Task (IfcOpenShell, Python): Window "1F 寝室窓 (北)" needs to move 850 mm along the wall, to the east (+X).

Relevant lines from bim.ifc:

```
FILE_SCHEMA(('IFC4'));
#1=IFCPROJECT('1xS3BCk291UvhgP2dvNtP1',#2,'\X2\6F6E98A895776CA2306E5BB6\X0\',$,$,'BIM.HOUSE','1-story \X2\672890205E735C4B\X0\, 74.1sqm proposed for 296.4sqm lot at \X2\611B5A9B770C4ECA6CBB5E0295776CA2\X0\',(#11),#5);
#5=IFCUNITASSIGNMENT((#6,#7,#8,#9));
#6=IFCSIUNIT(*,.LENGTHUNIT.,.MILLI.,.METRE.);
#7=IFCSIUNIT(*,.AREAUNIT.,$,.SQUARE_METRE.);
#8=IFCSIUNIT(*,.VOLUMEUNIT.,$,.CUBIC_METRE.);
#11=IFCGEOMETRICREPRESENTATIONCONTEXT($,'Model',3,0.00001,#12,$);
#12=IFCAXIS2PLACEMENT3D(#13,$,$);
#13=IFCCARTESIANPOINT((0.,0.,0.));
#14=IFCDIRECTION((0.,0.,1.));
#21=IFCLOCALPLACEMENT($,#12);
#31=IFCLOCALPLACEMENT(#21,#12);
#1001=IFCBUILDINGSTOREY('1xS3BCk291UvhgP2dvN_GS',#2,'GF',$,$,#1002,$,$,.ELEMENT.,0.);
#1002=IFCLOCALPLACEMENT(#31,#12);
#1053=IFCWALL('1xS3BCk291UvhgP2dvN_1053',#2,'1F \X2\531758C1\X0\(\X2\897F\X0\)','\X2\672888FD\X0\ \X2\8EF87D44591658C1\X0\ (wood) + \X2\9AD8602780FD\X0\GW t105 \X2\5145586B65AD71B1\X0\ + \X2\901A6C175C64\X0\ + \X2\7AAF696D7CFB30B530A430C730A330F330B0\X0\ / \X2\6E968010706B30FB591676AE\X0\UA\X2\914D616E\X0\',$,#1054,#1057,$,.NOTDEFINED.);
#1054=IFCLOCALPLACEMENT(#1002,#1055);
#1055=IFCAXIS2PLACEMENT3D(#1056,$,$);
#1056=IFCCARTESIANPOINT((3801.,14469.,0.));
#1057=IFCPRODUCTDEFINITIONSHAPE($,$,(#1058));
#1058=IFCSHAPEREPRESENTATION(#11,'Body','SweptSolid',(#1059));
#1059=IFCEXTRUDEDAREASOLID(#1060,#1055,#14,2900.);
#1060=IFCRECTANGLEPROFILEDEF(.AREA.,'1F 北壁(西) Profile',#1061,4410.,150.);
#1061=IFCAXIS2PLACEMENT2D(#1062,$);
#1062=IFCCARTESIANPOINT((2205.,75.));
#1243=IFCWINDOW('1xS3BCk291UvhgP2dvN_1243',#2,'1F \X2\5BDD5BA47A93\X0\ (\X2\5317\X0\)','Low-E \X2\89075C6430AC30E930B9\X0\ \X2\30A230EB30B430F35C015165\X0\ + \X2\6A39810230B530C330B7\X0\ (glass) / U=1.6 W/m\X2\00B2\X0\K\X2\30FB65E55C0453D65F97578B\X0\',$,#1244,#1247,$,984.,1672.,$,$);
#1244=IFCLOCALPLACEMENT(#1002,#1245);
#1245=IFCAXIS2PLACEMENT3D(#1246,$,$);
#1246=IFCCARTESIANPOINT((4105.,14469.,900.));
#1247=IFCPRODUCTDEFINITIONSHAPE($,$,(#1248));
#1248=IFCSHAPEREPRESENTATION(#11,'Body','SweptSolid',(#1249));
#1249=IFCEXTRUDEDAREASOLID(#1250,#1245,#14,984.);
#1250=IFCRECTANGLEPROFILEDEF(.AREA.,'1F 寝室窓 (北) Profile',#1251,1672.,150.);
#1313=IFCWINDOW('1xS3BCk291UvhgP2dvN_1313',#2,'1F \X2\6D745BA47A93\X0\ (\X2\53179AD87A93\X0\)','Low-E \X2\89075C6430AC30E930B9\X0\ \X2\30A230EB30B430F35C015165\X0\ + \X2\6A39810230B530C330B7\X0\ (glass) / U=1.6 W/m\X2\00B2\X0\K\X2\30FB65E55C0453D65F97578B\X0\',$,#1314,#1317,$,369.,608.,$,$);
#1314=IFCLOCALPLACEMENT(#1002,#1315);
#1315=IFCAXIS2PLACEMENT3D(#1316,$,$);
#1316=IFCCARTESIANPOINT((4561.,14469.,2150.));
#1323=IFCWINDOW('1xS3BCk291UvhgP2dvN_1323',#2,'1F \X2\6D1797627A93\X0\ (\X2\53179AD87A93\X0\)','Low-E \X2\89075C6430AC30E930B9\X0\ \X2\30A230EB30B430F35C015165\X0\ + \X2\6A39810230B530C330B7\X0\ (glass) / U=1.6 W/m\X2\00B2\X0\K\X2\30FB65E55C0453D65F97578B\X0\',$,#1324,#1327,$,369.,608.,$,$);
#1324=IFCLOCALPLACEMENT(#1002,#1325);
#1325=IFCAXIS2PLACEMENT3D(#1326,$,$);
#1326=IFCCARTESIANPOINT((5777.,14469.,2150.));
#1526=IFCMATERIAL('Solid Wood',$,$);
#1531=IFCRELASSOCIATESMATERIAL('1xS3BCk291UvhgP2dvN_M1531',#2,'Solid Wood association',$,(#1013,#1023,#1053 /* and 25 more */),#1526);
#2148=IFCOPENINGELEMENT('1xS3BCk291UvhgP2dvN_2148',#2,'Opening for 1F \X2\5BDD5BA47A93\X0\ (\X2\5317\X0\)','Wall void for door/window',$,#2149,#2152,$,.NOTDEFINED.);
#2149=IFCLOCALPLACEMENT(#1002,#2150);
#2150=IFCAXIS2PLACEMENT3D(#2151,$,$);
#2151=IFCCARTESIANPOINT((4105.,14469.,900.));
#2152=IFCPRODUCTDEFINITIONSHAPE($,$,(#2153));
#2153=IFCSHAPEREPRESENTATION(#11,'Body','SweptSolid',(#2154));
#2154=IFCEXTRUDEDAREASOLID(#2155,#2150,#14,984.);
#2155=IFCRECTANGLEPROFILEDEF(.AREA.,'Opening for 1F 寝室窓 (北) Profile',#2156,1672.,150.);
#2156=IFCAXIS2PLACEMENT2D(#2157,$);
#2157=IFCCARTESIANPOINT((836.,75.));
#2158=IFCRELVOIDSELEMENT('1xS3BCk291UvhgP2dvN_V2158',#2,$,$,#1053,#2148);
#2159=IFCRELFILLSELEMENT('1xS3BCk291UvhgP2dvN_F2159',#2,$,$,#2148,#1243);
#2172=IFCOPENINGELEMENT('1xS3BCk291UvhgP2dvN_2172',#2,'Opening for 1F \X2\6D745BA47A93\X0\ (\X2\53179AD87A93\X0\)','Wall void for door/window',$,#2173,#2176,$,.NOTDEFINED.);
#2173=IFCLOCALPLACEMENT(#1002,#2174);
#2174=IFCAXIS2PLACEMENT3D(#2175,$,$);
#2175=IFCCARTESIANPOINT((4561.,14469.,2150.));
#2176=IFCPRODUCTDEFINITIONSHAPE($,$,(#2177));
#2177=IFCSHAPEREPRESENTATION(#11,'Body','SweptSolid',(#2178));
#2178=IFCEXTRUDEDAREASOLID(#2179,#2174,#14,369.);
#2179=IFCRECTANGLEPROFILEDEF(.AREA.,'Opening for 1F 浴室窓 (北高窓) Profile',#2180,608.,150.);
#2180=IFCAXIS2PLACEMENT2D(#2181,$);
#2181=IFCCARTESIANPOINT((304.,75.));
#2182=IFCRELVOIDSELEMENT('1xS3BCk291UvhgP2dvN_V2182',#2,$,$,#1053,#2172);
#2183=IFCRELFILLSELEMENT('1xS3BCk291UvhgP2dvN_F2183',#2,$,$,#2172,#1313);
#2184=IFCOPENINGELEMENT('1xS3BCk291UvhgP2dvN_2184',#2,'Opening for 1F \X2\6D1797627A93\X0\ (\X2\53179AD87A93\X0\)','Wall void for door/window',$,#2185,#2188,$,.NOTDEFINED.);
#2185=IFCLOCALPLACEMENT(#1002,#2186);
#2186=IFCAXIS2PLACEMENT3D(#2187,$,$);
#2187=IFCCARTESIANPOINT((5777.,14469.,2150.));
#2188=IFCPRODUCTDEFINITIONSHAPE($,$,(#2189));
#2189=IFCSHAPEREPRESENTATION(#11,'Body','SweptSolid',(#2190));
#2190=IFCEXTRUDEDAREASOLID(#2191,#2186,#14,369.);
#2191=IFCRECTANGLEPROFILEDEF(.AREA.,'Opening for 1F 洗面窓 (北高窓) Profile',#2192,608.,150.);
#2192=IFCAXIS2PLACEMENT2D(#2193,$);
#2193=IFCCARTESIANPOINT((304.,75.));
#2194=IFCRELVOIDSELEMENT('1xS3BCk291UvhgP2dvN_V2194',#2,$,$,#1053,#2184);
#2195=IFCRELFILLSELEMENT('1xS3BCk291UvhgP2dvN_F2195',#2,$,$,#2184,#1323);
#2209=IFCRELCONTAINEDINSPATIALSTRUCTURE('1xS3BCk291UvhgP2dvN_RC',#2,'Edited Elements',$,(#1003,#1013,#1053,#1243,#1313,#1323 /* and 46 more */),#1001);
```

```python
import ifcopenshell
import ifcopenshell.api.geometry
import ifcopenshell.util.placement
import ifcopenshell.util.unit

model = ifcopenshell.open("bim.ifc")
unit_scale = ifcopenshell.util.unit.calculate_unit_scale(model)

window = model.by_id(1243)
opening = window.FillsVoids[0].RelatingOpeningElement
wall = opening.VoidsElements[0].RelatingBuildingElement

wall_matrix = ifcopenshell.util.placement.get_local_placement(wall.ObjectPlacement)
shift = wall_matrix[:3, 0] * 0.85 / unit_scale
before = ifcopenshell.util.placement.get_local_placement(window.ObjectPlacement)[:3, 3].copy()

# The window is not placed relative to its opening, so move both.
for product in (opening, window):
    matrix = ifcopenshell.util.placement.get_local_placement(product.ObjectPlacement)
    matrix[:3, 3] += shift
    ifcopenshell.api.geometry.edit_object_placement(model, product=product, matrix=matrix, is_si=False)

after = ifcopenshell.util.placement.get_local_placement(window.ObjectPlacement)[:3, 3]
print("window moved by", (after - before).round(3) + 0.0)

model.write("bim_updated.ifc")
```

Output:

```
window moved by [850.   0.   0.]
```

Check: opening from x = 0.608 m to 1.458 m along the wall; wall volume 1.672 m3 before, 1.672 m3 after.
